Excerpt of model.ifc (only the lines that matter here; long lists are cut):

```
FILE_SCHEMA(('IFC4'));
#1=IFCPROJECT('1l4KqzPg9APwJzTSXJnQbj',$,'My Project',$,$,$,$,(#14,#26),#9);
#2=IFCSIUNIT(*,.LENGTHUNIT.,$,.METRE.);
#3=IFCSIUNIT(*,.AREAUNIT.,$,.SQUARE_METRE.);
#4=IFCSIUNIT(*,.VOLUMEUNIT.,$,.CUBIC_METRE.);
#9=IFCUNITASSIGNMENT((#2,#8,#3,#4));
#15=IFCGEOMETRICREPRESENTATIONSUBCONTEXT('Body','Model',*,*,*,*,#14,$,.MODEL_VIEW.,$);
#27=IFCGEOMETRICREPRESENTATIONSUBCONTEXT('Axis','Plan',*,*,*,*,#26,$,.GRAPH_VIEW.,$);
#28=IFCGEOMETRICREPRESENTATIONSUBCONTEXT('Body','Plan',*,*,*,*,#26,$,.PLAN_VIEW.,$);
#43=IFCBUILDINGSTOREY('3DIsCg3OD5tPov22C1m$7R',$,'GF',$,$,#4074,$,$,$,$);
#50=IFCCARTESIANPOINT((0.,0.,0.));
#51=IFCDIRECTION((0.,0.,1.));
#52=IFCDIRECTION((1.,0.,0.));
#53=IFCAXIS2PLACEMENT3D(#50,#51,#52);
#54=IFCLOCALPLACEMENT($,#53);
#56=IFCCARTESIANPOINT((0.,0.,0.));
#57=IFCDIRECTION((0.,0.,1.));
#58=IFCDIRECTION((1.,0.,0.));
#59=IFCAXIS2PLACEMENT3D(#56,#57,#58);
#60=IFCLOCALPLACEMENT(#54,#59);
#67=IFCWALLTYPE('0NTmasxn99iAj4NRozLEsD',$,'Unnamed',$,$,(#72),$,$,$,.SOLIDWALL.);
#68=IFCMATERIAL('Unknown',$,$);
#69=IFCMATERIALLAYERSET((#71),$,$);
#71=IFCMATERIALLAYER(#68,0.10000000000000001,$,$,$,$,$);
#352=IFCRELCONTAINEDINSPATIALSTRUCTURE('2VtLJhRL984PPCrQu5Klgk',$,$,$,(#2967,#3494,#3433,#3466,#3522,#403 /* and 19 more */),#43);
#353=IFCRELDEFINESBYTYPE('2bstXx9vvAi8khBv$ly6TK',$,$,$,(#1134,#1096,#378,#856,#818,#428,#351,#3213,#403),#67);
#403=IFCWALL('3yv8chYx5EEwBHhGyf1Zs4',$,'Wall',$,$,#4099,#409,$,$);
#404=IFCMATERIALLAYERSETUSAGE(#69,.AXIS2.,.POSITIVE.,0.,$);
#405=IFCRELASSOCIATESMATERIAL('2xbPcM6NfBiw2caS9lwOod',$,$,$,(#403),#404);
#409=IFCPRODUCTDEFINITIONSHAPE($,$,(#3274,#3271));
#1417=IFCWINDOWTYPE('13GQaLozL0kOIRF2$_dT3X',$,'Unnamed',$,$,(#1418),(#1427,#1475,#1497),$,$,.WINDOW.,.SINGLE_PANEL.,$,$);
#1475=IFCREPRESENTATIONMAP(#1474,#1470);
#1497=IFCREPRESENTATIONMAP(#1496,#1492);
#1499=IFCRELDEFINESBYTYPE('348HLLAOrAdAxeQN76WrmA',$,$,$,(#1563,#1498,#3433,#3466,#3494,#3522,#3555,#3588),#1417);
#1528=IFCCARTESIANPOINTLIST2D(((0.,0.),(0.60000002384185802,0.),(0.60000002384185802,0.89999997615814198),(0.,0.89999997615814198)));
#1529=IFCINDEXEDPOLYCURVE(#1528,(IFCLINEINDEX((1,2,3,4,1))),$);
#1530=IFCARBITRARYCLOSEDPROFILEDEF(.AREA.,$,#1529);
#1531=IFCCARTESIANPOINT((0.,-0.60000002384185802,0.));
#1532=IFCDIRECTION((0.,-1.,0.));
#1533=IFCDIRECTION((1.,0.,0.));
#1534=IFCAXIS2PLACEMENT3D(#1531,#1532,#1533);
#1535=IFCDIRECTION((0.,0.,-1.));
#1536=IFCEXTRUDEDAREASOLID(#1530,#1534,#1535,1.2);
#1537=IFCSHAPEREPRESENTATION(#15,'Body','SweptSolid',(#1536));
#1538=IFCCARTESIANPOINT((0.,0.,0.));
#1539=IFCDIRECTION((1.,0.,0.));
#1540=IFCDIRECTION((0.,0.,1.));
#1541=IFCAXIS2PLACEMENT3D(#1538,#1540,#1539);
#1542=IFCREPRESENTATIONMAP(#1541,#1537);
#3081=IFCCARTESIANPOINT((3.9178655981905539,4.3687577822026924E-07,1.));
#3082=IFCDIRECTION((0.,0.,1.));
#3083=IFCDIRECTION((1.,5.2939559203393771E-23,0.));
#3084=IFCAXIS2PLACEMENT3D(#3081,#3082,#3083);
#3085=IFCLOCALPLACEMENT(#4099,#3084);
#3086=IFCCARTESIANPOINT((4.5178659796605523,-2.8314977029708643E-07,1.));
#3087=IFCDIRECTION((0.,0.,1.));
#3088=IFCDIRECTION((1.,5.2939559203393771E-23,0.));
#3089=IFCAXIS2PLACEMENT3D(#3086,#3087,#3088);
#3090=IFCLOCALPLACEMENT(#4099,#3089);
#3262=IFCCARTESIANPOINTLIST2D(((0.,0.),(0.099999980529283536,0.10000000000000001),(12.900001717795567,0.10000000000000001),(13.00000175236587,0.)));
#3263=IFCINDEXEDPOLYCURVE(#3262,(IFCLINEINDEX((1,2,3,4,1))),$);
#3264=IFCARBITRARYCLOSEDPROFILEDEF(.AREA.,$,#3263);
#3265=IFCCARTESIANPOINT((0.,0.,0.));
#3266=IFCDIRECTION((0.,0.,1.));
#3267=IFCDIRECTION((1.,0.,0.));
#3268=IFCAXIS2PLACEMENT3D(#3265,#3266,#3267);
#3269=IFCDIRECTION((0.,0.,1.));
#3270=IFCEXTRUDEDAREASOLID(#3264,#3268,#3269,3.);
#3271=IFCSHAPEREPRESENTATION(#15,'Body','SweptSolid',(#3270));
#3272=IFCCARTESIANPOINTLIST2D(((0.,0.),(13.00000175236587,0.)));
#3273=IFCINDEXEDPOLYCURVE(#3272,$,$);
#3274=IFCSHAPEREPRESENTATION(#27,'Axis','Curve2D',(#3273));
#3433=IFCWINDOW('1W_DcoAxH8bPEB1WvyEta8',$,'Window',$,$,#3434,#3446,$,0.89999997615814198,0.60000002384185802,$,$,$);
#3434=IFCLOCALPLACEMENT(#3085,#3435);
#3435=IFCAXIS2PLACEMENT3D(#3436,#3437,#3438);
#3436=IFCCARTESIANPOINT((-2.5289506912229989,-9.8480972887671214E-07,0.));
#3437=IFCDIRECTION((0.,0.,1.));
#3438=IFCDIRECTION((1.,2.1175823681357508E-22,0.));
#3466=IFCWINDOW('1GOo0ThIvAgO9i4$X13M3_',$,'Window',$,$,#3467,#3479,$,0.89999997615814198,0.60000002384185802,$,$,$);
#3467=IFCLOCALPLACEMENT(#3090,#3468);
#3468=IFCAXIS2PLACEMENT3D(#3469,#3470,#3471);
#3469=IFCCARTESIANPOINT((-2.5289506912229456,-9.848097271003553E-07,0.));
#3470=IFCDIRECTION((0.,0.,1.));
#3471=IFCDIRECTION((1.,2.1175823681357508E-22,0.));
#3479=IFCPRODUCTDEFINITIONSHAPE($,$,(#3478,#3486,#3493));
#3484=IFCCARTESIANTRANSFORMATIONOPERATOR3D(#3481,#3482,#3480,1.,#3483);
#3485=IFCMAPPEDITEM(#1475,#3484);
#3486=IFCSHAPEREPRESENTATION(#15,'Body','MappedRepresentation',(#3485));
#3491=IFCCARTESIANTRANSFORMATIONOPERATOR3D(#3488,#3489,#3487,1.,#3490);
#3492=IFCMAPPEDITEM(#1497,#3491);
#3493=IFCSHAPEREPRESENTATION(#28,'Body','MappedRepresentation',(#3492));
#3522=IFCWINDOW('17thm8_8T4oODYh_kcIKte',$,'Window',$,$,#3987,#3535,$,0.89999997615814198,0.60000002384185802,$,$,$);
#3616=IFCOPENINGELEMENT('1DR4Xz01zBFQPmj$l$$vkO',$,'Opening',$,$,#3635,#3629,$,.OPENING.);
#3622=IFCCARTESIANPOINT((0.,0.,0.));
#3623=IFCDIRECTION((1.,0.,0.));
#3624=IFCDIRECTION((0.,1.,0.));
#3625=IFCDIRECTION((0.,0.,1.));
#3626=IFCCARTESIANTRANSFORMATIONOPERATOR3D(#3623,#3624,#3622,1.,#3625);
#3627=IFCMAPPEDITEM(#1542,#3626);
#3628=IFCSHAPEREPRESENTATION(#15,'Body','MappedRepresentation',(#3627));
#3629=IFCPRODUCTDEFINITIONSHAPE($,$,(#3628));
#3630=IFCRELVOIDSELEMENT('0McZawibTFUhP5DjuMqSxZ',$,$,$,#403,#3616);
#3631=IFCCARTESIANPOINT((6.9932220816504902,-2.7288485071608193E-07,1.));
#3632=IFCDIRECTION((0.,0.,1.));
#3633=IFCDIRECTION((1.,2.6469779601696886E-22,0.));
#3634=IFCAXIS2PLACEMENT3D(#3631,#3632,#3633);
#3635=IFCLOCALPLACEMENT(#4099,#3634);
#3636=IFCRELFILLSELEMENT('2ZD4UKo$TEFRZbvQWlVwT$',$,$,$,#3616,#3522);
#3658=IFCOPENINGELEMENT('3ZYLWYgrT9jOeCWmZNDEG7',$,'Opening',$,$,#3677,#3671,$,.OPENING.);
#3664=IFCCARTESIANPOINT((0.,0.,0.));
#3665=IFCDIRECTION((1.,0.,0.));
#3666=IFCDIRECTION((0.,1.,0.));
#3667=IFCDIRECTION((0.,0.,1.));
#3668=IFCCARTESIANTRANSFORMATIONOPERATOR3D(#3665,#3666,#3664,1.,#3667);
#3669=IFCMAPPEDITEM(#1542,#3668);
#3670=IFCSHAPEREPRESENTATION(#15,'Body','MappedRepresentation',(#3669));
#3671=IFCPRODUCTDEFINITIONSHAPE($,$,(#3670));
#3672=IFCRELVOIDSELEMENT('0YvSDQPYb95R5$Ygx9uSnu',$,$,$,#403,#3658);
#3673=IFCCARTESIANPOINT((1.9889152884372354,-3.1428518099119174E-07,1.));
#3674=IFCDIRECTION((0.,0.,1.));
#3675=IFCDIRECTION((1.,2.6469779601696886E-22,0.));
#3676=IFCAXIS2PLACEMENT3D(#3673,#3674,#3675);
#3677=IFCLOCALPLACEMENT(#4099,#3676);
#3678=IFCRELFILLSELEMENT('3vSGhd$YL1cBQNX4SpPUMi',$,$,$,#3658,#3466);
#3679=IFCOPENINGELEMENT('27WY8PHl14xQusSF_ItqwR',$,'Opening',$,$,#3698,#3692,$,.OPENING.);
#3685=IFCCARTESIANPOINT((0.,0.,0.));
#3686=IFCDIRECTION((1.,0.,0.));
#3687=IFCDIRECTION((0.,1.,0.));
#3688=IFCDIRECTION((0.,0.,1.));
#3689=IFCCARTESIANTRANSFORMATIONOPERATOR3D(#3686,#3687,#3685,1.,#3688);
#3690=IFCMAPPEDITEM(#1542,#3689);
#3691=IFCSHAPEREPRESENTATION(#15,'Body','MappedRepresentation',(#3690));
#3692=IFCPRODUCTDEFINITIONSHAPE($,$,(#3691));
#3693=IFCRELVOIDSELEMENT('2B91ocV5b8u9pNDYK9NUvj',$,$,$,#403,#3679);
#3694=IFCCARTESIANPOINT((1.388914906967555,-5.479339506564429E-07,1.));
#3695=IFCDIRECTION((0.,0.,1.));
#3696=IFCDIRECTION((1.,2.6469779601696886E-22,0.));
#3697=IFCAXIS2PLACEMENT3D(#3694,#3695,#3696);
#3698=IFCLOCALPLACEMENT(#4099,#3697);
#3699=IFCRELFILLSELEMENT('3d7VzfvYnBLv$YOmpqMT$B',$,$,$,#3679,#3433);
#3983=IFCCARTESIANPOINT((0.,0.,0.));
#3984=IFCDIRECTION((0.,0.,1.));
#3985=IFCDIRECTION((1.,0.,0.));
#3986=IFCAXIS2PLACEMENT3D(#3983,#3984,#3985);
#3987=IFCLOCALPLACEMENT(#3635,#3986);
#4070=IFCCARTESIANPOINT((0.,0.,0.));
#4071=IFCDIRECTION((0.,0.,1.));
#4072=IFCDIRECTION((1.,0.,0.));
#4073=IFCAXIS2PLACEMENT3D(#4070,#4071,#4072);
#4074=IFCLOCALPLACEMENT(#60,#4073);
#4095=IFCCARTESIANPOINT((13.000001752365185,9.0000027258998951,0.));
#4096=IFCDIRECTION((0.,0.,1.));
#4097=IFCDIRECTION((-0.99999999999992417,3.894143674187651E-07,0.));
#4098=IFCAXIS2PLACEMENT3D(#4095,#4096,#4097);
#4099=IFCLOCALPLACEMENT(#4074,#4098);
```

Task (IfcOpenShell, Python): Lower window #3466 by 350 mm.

```python
import numpy as np
import ifcopenshell
import ifcopenshell.api.geometry
import ifcopenshell.util.placement
import ifcopenshell.util.unit

model = ifcopenshell.open("model.ifc")
unit_scale = ifcopenshell.util.unit.calculate_unit_scale(model)

window = model.by_guid("1GOo0ThIvAgO9i4$X13M3_")
opening = window.FillsVoids[0].RelatingOpeningElement
dz = -0.35

shift = np.array([0.0, 0.0, dz])
# The window is not placed relative to its opening, so move both.
for product in (opening, window):
    matrix = ifcopenshell.util.placement.get_local_placement(product.ObjectPlacement)
    matrix[:3, 3] += shift
    ifcopenshell.api.geometry.edit_object_placement(model, product=product, matrix=matrix, is_si=False)

print(f"moved by {dz * unit_scale:+.3f} m")

model.write("model-out.ifc")
```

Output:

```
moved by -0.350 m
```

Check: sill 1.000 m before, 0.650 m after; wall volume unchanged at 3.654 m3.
